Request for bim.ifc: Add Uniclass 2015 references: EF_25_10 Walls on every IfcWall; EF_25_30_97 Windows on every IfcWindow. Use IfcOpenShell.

First a look at what the model holds.

```python
import ifcopenshell

model = ifcopenshell.open("bim.ifc")
print(model.schema)
print("classifications:", [c.Name for c in model.by_type("IfcClassification")])
for ifc_class in ("IfcDoor", "IfcRoof", "IfcStair", "IfcWall", "IfcWindow"):
    print(ifc_class, len(model.by_type(ifc_class)))
```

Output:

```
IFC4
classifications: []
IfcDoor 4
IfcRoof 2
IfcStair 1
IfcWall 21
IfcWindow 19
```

```python
import ifcopenshell
import ifcopenshell.api.classification

model = ifcopenshell.open("bim.ifc")

system = ifcopenshell.api.classification.add_classification(model, classification="Uniclass 2015")

codes = {
    "IfcWall": ("EF_25_10", "Walls"),
    "IfcWindow": ("EF_25_30_97", "Windows"),
}
for ifc_class, (code, name) in codes.items():
    products = model.by_type(ifc_class)
    ifcopenshell.api.classification.add_reference(
        model, products=products, classification=system, identification=code, name=name
    )
    print(code, len(products))

model.write("bim_v2.ifc")
```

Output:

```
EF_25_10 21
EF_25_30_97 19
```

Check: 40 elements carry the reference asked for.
